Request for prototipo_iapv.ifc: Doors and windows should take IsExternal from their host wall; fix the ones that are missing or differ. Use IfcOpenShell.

First a look at what the model holds.

```python
import ifcopenshell
import ifcopenshell.util.element

model = ifcopenshell.open("prototipo_iapv.ifc")
print(model.schema)
seen = {}
for e in model.by_type("IfcDoor") + model.by_type("IfcWindow"):
    if not e.FillsVoids:
        continue
    host = e.FillsVoids[0].RelatingOpeningElement.VoidsElements[0].RelatingBuildingElement
    own = ifcopenshell.util.element.get_pset(e, f"Pset_{e.is_a()[3:].removesuffix('StandardCase')}Common", "IsExternal")
    wall = ifcopenshell.util.element.get_pset(host, "Pset_WallCommon", "IsExternal")
    seen[e.is_a(), own, wall] = seen.get((e.is_a(), own, wall), 0) + 1
for (cls, own, wall), count in sorted(seen.items(), key=str):
    print(count, cls, "IsExternal:", own, "| host wall:", wall)
```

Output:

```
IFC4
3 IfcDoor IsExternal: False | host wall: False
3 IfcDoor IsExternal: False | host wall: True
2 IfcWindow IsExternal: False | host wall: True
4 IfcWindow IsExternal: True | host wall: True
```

```python
import ifcopenshell
import ifcopenshell.api.pset
import ifcopenshell.util.element

model = ifcopenshell.open("prototipo_iapv.ifc")

count = 0
for ifc_class, pset_name in (("IfcDoor", "Pset_DoorCommon"), ("IfcWindow", "Pset_WindowCommon")):
    for e in model.by_type(ifc_class):
        if not e.FillsVoids:
            continue
        host = e.FillsVoids[0].RelatingOpeningElement.VoidsElements[0].RelatingBuildingElement
        external = ifcopenshell.util.element.get_pset(host, "Pset_WallCommon", "IsExternal")
        if external is None or ifcopenshell.util.element.get_pset(e, pset_name, "IsExternal") == external:
            continue
        pset = ifcopenshell.api.pset.add_pset(model, product=e, name=pset_name)
        ifcopenshell.api.pset.edit_pset(model, pset=pset, properties={"IsExternal": external})
        count += 1

print(count, "updated")

model.write("prototipo_iapv_updated.ifc")
```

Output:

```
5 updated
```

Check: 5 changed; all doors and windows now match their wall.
